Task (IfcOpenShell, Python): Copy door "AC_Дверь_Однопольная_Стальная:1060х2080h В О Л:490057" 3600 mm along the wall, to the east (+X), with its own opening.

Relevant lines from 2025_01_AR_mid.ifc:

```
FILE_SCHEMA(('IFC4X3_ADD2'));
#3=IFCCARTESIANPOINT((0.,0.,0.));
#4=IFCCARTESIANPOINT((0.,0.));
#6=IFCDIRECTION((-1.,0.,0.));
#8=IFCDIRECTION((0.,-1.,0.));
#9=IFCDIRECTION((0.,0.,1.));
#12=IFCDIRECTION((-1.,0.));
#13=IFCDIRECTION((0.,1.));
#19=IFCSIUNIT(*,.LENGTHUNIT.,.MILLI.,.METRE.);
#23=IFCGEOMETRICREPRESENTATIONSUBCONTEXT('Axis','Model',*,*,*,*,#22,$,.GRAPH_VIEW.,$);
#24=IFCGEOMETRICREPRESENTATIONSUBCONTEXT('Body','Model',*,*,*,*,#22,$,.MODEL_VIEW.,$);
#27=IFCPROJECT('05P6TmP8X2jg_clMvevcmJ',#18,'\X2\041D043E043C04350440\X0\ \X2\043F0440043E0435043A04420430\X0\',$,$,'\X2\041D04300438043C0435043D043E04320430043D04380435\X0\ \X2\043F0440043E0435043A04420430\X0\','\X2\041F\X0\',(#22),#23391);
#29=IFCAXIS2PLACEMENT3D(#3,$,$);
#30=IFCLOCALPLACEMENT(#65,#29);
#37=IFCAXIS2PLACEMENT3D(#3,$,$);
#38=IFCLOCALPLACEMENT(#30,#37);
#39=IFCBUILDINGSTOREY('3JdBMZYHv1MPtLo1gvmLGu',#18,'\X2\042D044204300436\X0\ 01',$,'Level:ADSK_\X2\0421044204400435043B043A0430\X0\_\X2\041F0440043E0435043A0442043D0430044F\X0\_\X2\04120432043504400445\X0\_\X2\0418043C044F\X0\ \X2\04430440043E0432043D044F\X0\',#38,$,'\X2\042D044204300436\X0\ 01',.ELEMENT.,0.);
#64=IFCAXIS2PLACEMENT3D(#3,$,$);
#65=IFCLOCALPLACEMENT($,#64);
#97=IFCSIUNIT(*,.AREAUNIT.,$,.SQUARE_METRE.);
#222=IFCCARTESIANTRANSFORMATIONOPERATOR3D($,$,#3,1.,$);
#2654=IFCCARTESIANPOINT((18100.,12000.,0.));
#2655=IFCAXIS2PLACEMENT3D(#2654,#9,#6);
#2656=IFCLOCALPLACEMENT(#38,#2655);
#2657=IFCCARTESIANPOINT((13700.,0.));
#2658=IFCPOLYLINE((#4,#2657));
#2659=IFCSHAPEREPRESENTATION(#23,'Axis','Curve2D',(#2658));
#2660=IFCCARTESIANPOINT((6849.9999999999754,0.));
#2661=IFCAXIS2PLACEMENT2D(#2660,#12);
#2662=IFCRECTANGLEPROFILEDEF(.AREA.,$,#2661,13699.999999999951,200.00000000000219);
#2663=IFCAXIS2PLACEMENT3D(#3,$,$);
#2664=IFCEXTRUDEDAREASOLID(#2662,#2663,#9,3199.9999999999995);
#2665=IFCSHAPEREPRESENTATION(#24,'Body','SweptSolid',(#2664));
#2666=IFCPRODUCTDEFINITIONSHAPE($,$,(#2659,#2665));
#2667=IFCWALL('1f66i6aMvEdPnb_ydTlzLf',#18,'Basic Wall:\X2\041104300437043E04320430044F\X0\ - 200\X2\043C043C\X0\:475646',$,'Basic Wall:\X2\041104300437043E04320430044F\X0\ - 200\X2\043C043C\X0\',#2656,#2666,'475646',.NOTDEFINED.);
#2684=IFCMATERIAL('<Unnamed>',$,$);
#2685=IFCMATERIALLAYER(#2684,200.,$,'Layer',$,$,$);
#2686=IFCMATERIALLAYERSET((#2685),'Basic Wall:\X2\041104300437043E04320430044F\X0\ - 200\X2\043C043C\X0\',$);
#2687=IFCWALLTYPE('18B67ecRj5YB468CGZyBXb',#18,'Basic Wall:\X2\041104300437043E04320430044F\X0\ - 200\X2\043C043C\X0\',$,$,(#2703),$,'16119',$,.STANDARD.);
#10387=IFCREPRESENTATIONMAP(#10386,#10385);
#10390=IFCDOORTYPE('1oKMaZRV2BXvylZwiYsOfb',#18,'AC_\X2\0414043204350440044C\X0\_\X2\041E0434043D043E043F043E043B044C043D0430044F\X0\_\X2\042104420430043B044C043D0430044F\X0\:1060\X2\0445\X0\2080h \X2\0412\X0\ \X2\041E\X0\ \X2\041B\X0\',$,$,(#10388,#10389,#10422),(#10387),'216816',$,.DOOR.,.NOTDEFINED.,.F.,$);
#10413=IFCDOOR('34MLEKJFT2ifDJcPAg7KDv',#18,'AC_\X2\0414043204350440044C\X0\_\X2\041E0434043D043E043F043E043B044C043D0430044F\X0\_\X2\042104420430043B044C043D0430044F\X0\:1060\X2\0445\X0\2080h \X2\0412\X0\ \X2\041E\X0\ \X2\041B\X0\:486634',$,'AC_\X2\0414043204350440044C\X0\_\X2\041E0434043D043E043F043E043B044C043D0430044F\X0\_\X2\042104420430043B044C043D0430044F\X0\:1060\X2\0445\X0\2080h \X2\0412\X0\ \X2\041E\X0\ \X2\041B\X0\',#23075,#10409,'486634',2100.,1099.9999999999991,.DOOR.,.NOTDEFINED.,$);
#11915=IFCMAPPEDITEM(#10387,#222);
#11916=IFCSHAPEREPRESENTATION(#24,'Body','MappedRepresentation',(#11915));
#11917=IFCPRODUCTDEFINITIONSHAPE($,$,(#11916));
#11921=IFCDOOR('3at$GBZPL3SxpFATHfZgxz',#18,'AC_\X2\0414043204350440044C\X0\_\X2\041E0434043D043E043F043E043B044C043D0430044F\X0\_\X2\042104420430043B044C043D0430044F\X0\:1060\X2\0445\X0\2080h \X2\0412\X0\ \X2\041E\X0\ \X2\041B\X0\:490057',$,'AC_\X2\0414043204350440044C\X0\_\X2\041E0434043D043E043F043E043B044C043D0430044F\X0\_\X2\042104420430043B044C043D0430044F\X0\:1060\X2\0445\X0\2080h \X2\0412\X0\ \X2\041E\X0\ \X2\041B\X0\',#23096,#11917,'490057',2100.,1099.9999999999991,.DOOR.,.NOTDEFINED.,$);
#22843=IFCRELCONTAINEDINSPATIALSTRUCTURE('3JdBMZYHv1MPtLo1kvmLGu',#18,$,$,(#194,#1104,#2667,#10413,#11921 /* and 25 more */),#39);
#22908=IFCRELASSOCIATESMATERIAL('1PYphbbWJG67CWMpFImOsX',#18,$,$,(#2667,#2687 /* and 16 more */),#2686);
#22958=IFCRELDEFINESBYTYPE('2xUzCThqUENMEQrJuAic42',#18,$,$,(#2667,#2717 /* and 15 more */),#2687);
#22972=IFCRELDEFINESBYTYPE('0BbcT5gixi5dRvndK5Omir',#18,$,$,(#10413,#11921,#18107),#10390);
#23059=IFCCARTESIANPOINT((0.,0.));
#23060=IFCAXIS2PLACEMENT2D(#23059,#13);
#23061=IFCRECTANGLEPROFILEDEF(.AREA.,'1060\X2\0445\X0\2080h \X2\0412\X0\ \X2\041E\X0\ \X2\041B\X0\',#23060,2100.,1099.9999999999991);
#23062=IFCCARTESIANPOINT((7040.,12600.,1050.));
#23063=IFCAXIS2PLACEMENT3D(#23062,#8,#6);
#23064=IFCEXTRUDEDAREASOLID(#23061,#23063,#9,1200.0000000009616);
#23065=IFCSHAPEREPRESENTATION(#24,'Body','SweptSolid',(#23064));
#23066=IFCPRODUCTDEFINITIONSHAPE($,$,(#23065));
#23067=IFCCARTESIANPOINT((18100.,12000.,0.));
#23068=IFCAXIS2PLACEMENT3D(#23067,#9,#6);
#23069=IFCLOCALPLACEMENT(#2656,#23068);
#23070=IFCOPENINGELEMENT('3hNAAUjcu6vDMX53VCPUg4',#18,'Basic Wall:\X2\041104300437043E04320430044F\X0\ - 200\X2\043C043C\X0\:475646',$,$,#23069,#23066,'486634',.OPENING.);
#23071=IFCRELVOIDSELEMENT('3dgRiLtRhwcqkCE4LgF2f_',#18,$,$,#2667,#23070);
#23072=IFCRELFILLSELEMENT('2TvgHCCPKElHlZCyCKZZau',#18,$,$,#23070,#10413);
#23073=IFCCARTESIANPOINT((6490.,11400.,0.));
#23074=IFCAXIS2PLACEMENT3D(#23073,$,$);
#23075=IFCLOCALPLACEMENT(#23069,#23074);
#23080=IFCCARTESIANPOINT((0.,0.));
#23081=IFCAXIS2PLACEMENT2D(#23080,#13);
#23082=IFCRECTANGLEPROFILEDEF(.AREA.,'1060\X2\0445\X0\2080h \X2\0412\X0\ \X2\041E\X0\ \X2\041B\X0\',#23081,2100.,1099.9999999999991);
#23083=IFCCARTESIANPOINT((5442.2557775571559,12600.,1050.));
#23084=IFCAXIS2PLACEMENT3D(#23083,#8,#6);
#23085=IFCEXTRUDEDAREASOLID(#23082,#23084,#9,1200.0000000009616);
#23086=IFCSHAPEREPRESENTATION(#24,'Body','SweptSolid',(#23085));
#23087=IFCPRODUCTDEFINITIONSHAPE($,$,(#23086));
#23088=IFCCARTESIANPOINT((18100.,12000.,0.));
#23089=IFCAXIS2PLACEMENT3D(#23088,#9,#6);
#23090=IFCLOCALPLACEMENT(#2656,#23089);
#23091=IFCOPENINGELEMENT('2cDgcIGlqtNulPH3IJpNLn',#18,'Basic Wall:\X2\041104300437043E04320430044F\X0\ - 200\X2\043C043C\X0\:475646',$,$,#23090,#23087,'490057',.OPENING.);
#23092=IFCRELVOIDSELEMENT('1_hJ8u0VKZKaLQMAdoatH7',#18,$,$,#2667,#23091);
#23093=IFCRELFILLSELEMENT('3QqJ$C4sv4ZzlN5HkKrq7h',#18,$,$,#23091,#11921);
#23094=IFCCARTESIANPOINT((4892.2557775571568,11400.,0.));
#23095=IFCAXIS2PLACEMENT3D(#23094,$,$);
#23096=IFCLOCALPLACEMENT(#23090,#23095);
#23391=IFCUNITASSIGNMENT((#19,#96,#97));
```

```python
import ifcopenshell
import ifcopenshell.api.feature
import ifcopenshell.api.geometry
import ifcopenshell.api.root
import ifcopenshell.geom
import ifcopenshell.util.element
import ifcopenshell.util.placement
import ifcopenshell.util.shape

model = ifcopenshell.open("2025_01_AR_mid.ifc")
settings = ifcopenshell.geom.settings()


def volume(element):
    """Net volume in cubic metres, openings subtracted."""
    shape = ifcopenshell.geom.create_shape(settings, element)
    return ifcopenshell.util.shape.get_volume(shape.geometry)


def reuse_history(source, copy):
    """copy_class also copies each property set's owner history, people and application; keep the originals."""
    for rel in copy.IsDefinedBy:
        if rel.is_a("IfcRelDefinesByProperties") and (history := rel.RelatingPropertyDefinition.OwnerHistory):
            rel.RelatingPropertyDefinition.OwnerHistory = source.OwnerHistory
            ifcopenshell.util.element.remove_deep2(model, history)


door = model.by_id(11921)
opening = door.FillsVoids[0].RelatingOpeningElement
wall = opening.VoidsElements[0].RelatingBuildingElement
before = volume(wall)
shift = ifcopenshell.util.placement.get_local_placement(wall.ObjectPlacement)[:3, 0] * -3600.0

# copy_class copies the void relationship, type, container and properties, but no geometry.
new_opening = ifcopenshell.api.root.copy_class(model, product=opening)
new_opening.Representation = ifcopenshell.util.element.copy_deep(
    model, opening.Representation, exclude=["IfcGeometricRepresentationContext", "IfcRepresentationMap"]
)
new_opening.Name = "Basic Wall:Базовая - 200мм"
new_opening.Tag = None
new_door = ifcopenshell.api.root.copy_class(model, product=door)
new_door.Representation = ifcopenshell.util.element.copy_deep(
    model, door.Representation, exclude=["IfcGeometricRepresentationContext", "IfcRepresentationMap"]
)
new_door.Name = "AC_Дверь_Однопольная_Стальная:1060х2080h В О Л"
new_door.Tag = None
reuse_history(door, new_door)
ifcopenshell.api.feature.add_filling(model, opening=new_opening, element=new_door)

for old, new in ((opening, new_opening), (door, new_door)):
    matrix = ifcopenshell.util.placement.get_local_placement(old.ObjectPlacement)
    matrix[:3, 3] += shift
    ifcopenshell.api.geometry.edit_object_placement(model, product=new, matrix=matrix, is_si=False)

after = volume(wall)

print(f"wall volume {before:.3f} -> {after:.3f} m3")

model.write("2025_01_AR_mid_updated.ifc")
```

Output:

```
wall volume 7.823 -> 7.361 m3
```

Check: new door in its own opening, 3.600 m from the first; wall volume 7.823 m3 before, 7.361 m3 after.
